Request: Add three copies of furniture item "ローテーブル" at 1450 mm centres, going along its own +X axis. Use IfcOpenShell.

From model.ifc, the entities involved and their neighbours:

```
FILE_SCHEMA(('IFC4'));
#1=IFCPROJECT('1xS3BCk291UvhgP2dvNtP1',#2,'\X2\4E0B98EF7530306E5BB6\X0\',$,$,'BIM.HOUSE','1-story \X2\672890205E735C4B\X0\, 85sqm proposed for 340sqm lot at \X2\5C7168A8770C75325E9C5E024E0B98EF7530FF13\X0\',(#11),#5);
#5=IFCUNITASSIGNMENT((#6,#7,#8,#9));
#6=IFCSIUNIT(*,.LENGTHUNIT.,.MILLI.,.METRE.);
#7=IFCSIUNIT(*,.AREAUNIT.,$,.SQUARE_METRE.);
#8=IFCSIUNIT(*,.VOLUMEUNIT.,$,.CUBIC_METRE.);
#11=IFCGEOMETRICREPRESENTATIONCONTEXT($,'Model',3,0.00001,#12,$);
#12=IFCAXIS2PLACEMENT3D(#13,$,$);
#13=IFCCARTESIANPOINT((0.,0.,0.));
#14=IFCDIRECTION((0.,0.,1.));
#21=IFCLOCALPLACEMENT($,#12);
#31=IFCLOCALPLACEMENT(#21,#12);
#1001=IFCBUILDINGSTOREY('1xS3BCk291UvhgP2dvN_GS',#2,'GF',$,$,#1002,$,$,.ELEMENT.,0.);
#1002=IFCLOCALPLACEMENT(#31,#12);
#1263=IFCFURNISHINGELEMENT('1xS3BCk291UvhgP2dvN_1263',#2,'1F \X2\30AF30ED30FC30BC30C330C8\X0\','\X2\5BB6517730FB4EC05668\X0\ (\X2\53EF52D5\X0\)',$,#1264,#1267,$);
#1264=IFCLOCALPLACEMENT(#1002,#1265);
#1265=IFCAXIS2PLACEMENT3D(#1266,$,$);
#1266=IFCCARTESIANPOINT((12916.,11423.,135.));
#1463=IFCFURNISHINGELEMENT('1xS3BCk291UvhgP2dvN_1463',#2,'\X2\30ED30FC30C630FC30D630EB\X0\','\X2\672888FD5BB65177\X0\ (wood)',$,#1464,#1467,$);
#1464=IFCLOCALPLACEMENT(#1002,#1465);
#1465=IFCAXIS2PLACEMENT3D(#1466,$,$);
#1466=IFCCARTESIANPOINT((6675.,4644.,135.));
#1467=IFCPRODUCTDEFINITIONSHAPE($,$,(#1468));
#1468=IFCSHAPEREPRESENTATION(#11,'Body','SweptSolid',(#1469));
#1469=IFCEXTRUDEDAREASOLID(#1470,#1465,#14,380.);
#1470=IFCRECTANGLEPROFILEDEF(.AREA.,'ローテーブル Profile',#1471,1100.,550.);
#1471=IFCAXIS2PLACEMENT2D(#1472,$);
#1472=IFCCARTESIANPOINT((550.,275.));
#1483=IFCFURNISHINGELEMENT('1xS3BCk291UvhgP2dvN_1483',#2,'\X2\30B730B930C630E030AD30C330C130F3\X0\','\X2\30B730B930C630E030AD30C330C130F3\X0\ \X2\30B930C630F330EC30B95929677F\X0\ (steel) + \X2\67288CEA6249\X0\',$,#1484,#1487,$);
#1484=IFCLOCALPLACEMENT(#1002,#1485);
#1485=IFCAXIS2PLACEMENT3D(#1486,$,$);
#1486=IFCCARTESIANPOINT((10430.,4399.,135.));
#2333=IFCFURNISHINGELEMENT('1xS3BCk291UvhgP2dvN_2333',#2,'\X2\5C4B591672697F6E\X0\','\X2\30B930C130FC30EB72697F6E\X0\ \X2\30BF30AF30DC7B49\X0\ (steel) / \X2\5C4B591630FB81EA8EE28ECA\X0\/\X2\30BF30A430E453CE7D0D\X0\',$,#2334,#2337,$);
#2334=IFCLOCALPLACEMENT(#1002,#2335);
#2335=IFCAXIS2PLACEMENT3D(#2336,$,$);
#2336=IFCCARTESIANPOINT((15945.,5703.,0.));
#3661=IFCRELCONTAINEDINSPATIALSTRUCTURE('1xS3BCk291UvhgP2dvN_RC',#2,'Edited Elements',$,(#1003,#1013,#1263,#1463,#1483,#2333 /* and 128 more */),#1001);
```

```python
import ifcopenshell
import ifcopenshell.api.geometry
import ifcopenshell.api.root
import ifcopenshell.util.element
import ifcopenshell.util.placement

model = ifcopenshell.open("model.ifc")


def reuse_history(source, copy):
    """copy_class also copies each property set's owner history, people and application; keep the originals."""
    for rel in copy.IsDefinedBy:
        if rel.is_a("IfcRelDefinesByProperties") and (history := rel.RelatingPropertyDefinition.OwnerHistory):
            rel.RelatingPropertyDefinition.OwnerHistory = source.OwnerHistory
            ifcopenshell.util.element.remove_deep2(model, history)


source = model.by_guid("1xS3BCk291UvhgP2dvN_1463")
base = ifcopenshell.util.placement.get_local_placement(source.ObjectPlacement)
step = base[:3, 0] * 1450.0

for i in range(1, 4):
    copy = ifcopenshell.api.root.copy_class(model, product=source)
    copy.Representation = ifcopenshell.util.element.copy_deep(
        model, source.Representation, exclude=["IfcGeometricRepresentationContext", "IfcRepresentationMap"]
    )
    reuse_history(source, copy)
    matrix = base.copy()
    matrix[:3, 3] += i * step
    print("added at", matrix[:3, 3].round(3) + 0.0)
    ifcopenshell.api.geometry.edit_object_placement(model, product=copy, matrix=matrix, is_si=False)

model.write("model_rev.ifc")
```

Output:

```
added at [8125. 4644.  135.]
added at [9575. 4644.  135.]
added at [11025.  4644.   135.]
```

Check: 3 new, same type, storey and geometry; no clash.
